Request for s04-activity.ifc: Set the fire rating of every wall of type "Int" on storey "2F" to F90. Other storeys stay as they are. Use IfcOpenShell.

First a look at what the model holds.

```python
import ifcopenshell
import ifcopenshell.util.element

model = ifcopenshell.open("s04-activity.ifc")
print(model.schema)
storey = next(s for s in model.by_type("IfcBuildingStorey") if s.Name == "2F")
walls = [e for e in ifcopenshell.util.element.get_decomposition(storey) if e.is_a("IfcWall")]
seen = {}
for e in walls:
    element_type = ifcopenshell.util.element.get_type(e)
    key = (element_type.Name if element_type != e and element_type else None, ifcopenshell.util.element.get_pset(e, "Pset_WallCommon", "FireRating"))
    seen[key] = seen.get(key, 0) + 1
for (name, value), count in sorted(seen.items(), key=str):
    print(count, "x", name, "|", value)
```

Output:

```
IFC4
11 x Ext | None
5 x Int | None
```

```python
import ifcopenshell
import ifcopenshell.api.pset
import ifcopenshell.util.element

model = ifcopenshell.open("s04-activity.ifc")

storey = next(s for s in model.by_type("IfcBuildingStorey") if s.Name == "2F")
walls = [e for e in ifcopenshell.util.element.get_decomposition(storey) if e.is_a("IfcWall")]

count = 0
for e in walls:
    element_type = ifcopenshell.util.element.get_type(e)
    if element_type in (None, e) or element_type.Name != "Int":
        continue
    # add_pset returns the element's existing set when there is one.
    pset = ifcopenshell.api.pset.add_pset(model, product=e, name="Pset_WallCommon")
    ifcopenshell.api.pset.edit_pset(model, pset=pset, properties={"FireRating": "F90"})
    count += 1

print(count, "walls updated")

model.write("s04-activity_rev.ifc")
```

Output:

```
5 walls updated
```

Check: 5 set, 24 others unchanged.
